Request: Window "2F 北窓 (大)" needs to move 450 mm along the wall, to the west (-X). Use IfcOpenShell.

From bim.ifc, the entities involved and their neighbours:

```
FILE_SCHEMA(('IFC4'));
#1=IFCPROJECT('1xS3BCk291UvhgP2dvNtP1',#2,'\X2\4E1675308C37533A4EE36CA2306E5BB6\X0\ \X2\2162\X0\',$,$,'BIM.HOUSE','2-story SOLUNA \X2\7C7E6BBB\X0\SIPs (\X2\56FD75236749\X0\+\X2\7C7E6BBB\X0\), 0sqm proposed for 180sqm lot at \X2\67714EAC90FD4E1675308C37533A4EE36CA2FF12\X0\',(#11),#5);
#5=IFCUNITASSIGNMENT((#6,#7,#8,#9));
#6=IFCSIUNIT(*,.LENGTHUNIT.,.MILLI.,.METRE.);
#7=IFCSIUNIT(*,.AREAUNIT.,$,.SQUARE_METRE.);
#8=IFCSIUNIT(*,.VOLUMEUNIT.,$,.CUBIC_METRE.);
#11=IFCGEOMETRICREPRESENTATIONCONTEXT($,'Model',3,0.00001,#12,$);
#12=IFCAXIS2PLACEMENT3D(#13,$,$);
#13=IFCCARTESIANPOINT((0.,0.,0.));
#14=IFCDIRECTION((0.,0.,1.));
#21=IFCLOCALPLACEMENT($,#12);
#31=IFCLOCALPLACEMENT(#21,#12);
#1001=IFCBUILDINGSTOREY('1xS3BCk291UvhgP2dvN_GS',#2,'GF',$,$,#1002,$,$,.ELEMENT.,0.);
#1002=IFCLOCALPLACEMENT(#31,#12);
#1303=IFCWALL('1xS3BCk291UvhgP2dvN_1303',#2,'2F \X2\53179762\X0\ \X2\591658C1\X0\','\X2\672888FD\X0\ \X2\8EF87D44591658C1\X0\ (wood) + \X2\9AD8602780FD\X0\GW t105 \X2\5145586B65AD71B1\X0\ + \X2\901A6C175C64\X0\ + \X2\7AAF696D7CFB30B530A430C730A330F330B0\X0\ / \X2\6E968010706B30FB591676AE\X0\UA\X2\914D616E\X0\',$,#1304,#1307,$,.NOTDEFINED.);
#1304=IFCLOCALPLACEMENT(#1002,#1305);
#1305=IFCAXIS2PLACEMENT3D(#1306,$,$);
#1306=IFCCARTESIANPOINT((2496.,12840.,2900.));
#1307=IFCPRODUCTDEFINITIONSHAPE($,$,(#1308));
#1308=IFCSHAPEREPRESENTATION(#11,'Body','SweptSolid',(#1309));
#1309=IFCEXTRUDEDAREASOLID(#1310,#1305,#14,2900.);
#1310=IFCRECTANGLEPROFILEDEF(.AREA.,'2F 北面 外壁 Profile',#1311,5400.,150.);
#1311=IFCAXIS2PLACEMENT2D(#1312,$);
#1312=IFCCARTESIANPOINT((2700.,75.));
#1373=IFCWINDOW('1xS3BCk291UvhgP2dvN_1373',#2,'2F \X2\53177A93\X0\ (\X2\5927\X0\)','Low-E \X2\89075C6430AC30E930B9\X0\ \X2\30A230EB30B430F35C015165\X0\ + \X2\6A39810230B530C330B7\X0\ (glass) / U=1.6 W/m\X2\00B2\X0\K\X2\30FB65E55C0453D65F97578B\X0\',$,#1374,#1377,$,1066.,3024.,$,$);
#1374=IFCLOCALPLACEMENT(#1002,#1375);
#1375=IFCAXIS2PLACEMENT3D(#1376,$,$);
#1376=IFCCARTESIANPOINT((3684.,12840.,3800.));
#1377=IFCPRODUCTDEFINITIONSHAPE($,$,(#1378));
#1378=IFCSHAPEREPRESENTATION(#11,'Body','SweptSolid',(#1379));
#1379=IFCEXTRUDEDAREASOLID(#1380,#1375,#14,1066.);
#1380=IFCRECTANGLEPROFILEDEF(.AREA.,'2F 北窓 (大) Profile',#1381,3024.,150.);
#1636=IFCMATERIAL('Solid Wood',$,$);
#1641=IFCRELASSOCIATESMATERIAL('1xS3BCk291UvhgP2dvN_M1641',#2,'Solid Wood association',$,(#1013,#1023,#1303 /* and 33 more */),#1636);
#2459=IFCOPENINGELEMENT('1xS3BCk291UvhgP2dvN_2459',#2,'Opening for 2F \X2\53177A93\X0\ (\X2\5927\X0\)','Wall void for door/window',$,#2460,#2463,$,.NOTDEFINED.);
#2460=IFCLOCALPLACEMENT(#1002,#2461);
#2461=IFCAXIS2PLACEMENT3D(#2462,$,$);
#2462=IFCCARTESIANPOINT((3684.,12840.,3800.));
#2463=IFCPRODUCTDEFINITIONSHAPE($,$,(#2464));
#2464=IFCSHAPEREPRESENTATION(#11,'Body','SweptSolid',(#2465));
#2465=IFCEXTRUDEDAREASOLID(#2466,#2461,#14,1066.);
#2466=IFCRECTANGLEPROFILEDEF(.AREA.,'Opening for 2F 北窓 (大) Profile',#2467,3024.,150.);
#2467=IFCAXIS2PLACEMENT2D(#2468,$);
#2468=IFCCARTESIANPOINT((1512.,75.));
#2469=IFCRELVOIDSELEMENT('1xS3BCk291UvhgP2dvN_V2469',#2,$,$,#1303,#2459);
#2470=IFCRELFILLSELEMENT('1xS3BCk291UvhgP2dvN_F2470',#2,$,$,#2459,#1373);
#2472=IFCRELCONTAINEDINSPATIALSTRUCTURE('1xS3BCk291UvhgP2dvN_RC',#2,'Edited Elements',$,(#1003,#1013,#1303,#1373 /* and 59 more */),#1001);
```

```python
import ifcopenshell
import ifcopenshell.api.geometry
import ifcopenshell.util.placement
import ifcopenshell.util.unit

model = ifcopenshell.open("bim.ifc")
unit_scale = ifcopenshell.util.unit.calculate_unit_scale(model)

window = model.by_id(1373)
opening = window.FillsVoids[0].RelatingOpeningElement
wall = opening.VoidsElements[0].RelatingBuildingElement

wall_matrix = ifcopenshell.util.placement.get_local_placement(wall.ObjectPlacement)
shift = wall_matrix[:3, 0] * -0.45 / unit_scale
before = ifcopenshell.util.placement.get_local_placement(window.ObjectPlacement)[:3, 3].copy()

# The window is not placed relative to its opening, so move both.
for product in (opening, window):
    matrix = ifcopenshell.util.placement.get_local_placement(product.ObjectPlacement)
    matrix[:3, 3] += shift
    ifcopenshell.api.geometry.edit_object_placement(model, product=product, matrix=matrix, is_si=False)

after = ifcopenshell.util.placement.get_local_placement(window.ObjectPlacement)[:3, 3]
print("window moved by", (after - before).round(3) + 0.0)

model.write("bim_updated.ifc")
```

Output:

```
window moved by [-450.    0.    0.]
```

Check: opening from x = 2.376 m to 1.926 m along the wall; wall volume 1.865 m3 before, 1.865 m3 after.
